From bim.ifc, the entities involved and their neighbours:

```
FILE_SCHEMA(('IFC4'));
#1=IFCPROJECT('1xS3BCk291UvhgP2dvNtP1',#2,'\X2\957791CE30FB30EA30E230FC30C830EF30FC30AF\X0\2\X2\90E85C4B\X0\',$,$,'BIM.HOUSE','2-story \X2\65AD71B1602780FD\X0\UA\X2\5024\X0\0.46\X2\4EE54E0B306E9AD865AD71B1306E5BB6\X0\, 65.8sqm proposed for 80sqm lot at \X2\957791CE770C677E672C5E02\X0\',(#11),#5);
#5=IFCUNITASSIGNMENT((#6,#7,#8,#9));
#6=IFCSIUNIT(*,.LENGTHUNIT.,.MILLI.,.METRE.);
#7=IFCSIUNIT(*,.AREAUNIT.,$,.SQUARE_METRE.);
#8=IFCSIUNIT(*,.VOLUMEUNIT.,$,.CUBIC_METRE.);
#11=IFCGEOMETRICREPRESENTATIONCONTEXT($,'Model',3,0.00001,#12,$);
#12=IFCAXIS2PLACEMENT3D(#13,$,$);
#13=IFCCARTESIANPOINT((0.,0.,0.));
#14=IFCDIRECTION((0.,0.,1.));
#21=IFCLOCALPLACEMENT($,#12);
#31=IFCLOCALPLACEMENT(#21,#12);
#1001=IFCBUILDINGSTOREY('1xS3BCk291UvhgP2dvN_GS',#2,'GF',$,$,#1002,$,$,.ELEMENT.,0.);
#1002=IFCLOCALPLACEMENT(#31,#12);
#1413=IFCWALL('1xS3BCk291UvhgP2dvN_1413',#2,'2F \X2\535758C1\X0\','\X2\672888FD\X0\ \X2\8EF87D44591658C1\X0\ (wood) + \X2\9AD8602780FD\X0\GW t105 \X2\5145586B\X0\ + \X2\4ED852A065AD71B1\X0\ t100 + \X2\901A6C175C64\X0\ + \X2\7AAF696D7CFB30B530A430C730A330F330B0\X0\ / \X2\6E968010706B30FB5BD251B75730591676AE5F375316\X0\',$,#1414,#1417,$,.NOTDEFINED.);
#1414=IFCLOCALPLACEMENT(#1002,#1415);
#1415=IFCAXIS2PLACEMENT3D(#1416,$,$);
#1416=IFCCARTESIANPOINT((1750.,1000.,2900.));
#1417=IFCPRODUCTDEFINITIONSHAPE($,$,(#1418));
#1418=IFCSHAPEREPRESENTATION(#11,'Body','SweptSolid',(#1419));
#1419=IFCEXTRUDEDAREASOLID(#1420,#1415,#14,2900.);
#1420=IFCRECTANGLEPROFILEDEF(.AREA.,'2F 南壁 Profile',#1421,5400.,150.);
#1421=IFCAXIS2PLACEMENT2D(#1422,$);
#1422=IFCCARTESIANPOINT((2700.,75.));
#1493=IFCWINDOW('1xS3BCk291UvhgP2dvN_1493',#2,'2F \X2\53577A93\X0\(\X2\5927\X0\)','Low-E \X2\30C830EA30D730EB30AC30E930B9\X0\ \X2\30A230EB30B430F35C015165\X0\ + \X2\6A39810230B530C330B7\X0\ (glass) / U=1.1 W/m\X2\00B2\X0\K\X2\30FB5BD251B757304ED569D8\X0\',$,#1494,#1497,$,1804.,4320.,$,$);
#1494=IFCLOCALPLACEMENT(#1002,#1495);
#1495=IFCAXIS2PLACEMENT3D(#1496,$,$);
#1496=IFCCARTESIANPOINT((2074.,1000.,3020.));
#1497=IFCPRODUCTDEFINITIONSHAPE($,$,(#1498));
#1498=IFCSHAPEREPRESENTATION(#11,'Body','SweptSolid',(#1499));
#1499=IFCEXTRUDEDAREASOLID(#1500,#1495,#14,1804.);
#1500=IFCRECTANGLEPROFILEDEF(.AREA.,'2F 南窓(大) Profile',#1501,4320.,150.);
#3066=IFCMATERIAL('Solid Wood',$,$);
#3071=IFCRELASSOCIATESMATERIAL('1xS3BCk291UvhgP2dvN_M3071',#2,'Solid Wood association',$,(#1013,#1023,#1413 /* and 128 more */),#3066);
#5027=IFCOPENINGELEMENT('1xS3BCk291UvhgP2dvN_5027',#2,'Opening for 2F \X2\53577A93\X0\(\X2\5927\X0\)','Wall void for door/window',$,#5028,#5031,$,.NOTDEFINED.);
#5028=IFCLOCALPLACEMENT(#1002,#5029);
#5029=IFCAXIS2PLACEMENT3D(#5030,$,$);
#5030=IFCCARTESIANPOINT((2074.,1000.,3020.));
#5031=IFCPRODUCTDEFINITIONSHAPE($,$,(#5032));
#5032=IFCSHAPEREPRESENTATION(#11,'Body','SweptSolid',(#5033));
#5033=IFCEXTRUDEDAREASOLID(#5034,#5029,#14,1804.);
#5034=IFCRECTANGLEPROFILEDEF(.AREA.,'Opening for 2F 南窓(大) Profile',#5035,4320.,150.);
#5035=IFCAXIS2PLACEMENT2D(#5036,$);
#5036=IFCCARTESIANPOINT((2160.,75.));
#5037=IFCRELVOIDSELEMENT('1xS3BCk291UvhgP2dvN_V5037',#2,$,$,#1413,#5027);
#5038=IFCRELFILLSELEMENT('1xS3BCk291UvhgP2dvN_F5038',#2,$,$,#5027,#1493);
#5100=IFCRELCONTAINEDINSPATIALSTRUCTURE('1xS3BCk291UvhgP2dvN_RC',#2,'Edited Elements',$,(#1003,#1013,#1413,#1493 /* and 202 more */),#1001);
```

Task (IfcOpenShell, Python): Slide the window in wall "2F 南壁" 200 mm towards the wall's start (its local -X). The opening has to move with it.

```python
import ifcopenshell
import ifcopenshell.api.geometry
import ifcopenshell.util.placement
import ifcopenshell.util.unit

model = ifcopenshell.open("bim.ifc")
unit_scale = ifcopenshell.util.unit.calculate_unit_scale(model)

window = model.by_guid("1xS3BCk291UvhgP2dvN_1493")
opening = window.FillsVoids[0].RelatingOpeningElement
wall = opening.VoidsElements[0].RelatingBuildingElement

wall_matrix = ifcopenshell.util.placement.get_local_placement(wall.ObjectPlacement)
shift = wall_matrix[:3, 0] * -0.2 / unit_scale
before = ifcopenshell.util.placement.get_local_placement(window.ObjectPlacement)[:3, 3].copy()

# The window is not placed relative to its opening, so move both.
for product in (opening, window):
    matrix = ifcopenshell.util.placement.get_local_placement(product.ObjectPlacement)
    matrix[:3, 3] += shift
    ifcopenshell.api.geometry.edit_object_placement(model, product=product, matrix=matrix, is_si=False)

after = ifcopenshell.util.placement.get_local_placement(window.ObjectPlacement)[:3, 3]
print("window moved by", (after - before).round(3) + 0.0)

model.write("bim_edited.ifc")
```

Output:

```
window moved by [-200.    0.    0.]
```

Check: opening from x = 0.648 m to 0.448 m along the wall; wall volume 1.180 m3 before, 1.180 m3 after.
